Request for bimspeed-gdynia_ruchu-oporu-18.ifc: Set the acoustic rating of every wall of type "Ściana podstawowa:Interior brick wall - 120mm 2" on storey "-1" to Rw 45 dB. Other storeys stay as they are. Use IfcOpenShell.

First a look at what the model holds.

```python
import ifcopenshell
import ifcopenshell.util.element

model = ifcopenshell.open("bimspeed-gdynia_ruchu-oporu-18.ifc")
print(model.schema)
storey = next(s for s in model.by_type("IfcBuildingStorey") if s.Name == "-1")
walls = [e for e in ifcopenshell.util.element.get_decomposition(storey) if e.is_a("IfcWall")]
seen = {}
for e in walls:
    element_type = ifcopenshell.util.element.get_type(e)
    key = (element_type.Name if element_type != e and element_type else None, ifcopenshell.util.element.get_pset(e, "Pset_WallCommon", "AcousticRating"))
    seen[key] = seen.get(key, 0) + 1
for (name, value), count in sorted(seen.items(), key=str):
    print(count, "x", name, "|", value)
```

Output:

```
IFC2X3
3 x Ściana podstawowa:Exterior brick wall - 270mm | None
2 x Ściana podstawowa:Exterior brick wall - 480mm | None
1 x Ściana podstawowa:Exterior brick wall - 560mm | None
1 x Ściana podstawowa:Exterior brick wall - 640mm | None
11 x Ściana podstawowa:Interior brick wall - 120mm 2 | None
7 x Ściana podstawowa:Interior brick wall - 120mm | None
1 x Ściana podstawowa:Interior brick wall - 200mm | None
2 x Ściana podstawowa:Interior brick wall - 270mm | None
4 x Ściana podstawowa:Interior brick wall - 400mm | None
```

```python
import ifcopenshell
import ifcopenshell.api.pset
import ifcopenshell.util.element

model = ifcopenshell.open("bimspeed-gdynia_ruchu-oporu-18.ifc")

storey = next(s for s in model.by_type("IfcBuildingStorey") if s.Name == "-1")
walls = [e for e in ifcopenshell.util.element.get_decomposition(storey) if e.is_a("IfcWall")]

count = 0
for e in walls:
    element_type = ifcopenshell.util.element.get_type(e)
    if element_type in (None, e) or element_type.Name != "Ściana podstawowa:Interior brick wall - 120mm 2":
        continue
    # add_pset returns the element's existing set when there is one.
    pset = ifcopenshell.api.pset.add_pset(model, product=e, name="Pset_WallCommon")
    ifcopenshell.api.pset.edit_pset(model, pset=pset, properties={"AcousticRating": "Rw 45 dB"})
    count += 1

print(count, "walls updated")

model.write("bimspeed-gdynia_ruchu-oporu-18-out.ifc")
```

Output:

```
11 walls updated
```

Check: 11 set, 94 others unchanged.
